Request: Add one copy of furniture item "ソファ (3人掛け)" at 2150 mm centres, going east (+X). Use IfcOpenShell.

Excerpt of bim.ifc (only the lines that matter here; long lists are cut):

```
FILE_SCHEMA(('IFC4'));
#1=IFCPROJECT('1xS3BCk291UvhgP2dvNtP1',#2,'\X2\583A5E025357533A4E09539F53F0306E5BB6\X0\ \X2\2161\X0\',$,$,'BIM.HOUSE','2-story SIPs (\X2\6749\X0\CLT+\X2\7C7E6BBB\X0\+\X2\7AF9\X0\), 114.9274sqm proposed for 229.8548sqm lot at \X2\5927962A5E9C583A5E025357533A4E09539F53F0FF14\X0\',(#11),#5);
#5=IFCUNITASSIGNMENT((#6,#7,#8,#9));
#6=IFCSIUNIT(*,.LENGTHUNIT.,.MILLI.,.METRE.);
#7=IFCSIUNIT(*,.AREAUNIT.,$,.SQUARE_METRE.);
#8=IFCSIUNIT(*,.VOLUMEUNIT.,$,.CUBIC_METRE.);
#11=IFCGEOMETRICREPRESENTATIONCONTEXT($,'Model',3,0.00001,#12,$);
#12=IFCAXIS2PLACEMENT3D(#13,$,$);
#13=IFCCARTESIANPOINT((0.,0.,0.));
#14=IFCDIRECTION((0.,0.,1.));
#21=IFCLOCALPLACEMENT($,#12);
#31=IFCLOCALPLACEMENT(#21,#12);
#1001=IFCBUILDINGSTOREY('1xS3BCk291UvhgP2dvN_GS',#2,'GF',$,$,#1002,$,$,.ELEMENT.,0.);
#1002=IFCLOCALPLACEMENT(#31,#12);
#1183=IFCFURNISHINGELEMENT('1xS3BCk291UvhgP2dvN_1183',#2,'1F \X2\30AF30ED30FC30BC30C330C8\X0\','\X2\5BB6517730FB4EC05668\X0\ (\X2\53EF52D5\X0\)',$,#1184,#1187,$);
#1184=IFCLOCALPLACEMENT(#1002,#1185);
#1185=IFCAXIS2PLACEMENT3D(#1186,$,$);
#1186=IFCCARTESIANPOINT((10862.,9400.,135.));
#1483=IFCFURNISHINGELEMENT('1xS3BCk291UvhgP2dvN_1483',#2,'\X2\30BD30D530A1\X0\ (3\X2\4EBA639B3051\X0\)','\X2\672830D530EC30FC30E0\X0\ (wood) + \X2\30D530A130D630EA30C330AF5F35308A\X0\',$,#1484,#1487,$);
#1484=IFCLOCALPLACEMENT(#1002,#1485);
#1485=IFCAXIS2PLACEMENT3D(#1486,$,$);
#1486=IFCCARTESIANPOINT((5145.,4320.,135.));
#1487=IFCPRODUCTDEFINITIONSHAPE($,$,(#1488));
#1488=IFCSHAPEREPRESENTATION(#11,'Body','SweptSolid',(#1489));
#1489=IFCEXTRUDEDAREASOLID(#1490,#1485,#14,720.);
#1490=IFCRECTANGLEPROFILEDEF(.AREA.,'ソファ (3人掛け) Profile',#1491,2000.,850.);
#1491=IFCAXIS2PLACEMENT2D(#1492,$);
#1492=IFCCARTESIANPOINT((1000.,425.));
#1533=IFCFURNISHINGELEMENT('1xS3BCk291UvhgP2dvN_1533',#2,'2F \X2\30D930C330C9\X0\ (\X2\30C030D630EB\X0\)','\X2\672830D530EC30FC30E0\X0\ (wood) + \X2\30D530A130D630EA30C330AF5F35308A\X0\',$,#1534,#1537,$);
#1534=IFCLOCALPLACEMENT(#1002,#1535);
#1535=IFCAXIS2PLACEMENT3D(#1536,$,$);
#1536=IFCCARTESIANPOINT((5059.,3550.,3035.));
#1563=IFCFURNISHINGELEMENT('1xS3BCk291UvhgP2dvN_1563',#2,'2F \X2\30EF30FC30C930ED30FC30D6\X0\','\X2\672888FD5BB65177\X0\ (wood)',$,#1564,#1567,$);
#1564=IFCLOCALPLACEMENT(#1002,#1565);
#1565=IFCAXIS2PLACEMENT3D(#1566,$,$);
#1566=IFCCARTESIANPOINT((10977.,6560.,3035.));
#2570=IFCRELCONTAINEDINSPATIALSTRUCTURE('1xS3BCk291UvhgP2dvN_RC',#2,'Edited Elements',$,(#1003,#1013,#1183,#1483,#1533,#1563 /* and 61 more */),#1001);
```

```python
import numpy as np
import ifcopenshell
import ifcopenshell.api.geometry
import ifcopenshell.api.root
import ifcopenshell.util.element
import ifcopenshell.util.placement

model = ifcopenshell.open("bim.ifc")


def reuse_history(source, copy):
    """copy_class also copies each property set's owner history, people and application; keep the originals."""
    for rel in copy.IsDefinedBy:
        if rel.is_a("IfcRelDefinesByProperties") and (history := rel.RelatingPropertyDefinition.OwnerHistory):
            rel.RelatingPropertyDefinition.OwnerHistory = source.OwnerHistory
            ifcopenshell.util.element.remove_deep2(model, history)


source = model.by_guid("1xS3BCk291UvhgP2dvN_1483")
base = ifcopenshell.util.placement.get_local_placement(source.ObjectPlacement)
step = np.array([1.0, 0.0, 0.0]) * 2150.0

for i in range(1, 2):
    copy = ifcopenshell.api.root.copy_class(model, product=source)
    copy.Representation = ifcopenshell.util.element.copy_deep(
        model, source.Representation, exclude=["IfcGeometricRepresentationContext", "IfcRepresentationMap"]
    )
    reuse_history(source, copy)
    matrix = base.copy()
    matrix[:3, 3] += i * step
    print("added at", matrix[:3, 3].round(3) + 0.0)
    ifcopenshell.api.geometry.edit_object_placement(model, product=copy, matrix=matrix, is_si=False)

model.write("bim_v2.ifc")
```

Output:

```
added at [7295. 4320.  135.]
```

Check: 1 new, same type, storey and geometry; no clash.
